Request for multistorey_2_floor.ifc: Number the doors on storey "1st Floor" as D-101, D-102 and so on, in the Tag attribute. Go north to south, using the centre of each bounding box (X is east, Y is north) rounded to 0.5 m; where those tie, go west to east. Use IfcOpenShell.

First a look at what the model holds.

```python
import ifcopenshell
import ifcopenshell.util.element
import ifcopenshell.util.placement

model = ifcopenshell.open("multistorey_2_floor.ifc")
print(model.schema)
storey = next(s for s in model.by_type("IfcBuildingStorey") if s.Name == "1st Floor")
doors = [e for e in ifcopenshell.util.element.get_decomposition(storey) if e.is_a("IfcDoor")]
for e in sorted(doors, key=lambda e: e.id()):
    origin = ifcopenshell.util.placement.get_local_placement(e.ObjectPlacement)[:3, 3]
    print(e.id(), e.Tag, e.Name, origin.round(2) + 0.0, sep=" | ")
```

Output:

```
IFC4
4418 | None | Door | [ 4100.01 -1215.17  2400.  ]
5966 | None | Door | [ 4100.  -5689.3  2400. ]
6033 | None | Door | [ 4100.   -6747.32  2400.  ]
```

```python
import ifcopenshell
import ifcopenshell.geom
import ifcopenshell.util.element
import ifcopenshell.util.shape

model = ifcopenshell.open("multistorey_2_floor.ifc")
settings = ifcopenshell.geom.settings()
settings.set("use-world-coords", True)


def centre(element):
    shape = ifcopenshell.geom.create_shape(settings, element)
    return ifcopenshell.util.shape.get_bbox_centroid(shape.geometry)


storey = next(s for s in model.by_type("IfcBuildingStorey") if s.Name == "1st Floor")
doors = [e for e in ifcopenshell.util.element.get_decomposition(storey) if e.is_a("IfcDoor")]

# Insertion points can sit at a corner or the storey origin, so sort by the geometry (in metres).
centres = {e: centre(e) for e in doors}
doors.sort(key=lambda e: (-round(centres[e][1] / 0.5), centres[e][0]))

for i, e in enumerate(doors, start=1):
    number = f"D-1{i:02d}"
    e.Tag = number
    print(e.id(), number)

model.write("multistorey_2_floor_v2.ifc")
```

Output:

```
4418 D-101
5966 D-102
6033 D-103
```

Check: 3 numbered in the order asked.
